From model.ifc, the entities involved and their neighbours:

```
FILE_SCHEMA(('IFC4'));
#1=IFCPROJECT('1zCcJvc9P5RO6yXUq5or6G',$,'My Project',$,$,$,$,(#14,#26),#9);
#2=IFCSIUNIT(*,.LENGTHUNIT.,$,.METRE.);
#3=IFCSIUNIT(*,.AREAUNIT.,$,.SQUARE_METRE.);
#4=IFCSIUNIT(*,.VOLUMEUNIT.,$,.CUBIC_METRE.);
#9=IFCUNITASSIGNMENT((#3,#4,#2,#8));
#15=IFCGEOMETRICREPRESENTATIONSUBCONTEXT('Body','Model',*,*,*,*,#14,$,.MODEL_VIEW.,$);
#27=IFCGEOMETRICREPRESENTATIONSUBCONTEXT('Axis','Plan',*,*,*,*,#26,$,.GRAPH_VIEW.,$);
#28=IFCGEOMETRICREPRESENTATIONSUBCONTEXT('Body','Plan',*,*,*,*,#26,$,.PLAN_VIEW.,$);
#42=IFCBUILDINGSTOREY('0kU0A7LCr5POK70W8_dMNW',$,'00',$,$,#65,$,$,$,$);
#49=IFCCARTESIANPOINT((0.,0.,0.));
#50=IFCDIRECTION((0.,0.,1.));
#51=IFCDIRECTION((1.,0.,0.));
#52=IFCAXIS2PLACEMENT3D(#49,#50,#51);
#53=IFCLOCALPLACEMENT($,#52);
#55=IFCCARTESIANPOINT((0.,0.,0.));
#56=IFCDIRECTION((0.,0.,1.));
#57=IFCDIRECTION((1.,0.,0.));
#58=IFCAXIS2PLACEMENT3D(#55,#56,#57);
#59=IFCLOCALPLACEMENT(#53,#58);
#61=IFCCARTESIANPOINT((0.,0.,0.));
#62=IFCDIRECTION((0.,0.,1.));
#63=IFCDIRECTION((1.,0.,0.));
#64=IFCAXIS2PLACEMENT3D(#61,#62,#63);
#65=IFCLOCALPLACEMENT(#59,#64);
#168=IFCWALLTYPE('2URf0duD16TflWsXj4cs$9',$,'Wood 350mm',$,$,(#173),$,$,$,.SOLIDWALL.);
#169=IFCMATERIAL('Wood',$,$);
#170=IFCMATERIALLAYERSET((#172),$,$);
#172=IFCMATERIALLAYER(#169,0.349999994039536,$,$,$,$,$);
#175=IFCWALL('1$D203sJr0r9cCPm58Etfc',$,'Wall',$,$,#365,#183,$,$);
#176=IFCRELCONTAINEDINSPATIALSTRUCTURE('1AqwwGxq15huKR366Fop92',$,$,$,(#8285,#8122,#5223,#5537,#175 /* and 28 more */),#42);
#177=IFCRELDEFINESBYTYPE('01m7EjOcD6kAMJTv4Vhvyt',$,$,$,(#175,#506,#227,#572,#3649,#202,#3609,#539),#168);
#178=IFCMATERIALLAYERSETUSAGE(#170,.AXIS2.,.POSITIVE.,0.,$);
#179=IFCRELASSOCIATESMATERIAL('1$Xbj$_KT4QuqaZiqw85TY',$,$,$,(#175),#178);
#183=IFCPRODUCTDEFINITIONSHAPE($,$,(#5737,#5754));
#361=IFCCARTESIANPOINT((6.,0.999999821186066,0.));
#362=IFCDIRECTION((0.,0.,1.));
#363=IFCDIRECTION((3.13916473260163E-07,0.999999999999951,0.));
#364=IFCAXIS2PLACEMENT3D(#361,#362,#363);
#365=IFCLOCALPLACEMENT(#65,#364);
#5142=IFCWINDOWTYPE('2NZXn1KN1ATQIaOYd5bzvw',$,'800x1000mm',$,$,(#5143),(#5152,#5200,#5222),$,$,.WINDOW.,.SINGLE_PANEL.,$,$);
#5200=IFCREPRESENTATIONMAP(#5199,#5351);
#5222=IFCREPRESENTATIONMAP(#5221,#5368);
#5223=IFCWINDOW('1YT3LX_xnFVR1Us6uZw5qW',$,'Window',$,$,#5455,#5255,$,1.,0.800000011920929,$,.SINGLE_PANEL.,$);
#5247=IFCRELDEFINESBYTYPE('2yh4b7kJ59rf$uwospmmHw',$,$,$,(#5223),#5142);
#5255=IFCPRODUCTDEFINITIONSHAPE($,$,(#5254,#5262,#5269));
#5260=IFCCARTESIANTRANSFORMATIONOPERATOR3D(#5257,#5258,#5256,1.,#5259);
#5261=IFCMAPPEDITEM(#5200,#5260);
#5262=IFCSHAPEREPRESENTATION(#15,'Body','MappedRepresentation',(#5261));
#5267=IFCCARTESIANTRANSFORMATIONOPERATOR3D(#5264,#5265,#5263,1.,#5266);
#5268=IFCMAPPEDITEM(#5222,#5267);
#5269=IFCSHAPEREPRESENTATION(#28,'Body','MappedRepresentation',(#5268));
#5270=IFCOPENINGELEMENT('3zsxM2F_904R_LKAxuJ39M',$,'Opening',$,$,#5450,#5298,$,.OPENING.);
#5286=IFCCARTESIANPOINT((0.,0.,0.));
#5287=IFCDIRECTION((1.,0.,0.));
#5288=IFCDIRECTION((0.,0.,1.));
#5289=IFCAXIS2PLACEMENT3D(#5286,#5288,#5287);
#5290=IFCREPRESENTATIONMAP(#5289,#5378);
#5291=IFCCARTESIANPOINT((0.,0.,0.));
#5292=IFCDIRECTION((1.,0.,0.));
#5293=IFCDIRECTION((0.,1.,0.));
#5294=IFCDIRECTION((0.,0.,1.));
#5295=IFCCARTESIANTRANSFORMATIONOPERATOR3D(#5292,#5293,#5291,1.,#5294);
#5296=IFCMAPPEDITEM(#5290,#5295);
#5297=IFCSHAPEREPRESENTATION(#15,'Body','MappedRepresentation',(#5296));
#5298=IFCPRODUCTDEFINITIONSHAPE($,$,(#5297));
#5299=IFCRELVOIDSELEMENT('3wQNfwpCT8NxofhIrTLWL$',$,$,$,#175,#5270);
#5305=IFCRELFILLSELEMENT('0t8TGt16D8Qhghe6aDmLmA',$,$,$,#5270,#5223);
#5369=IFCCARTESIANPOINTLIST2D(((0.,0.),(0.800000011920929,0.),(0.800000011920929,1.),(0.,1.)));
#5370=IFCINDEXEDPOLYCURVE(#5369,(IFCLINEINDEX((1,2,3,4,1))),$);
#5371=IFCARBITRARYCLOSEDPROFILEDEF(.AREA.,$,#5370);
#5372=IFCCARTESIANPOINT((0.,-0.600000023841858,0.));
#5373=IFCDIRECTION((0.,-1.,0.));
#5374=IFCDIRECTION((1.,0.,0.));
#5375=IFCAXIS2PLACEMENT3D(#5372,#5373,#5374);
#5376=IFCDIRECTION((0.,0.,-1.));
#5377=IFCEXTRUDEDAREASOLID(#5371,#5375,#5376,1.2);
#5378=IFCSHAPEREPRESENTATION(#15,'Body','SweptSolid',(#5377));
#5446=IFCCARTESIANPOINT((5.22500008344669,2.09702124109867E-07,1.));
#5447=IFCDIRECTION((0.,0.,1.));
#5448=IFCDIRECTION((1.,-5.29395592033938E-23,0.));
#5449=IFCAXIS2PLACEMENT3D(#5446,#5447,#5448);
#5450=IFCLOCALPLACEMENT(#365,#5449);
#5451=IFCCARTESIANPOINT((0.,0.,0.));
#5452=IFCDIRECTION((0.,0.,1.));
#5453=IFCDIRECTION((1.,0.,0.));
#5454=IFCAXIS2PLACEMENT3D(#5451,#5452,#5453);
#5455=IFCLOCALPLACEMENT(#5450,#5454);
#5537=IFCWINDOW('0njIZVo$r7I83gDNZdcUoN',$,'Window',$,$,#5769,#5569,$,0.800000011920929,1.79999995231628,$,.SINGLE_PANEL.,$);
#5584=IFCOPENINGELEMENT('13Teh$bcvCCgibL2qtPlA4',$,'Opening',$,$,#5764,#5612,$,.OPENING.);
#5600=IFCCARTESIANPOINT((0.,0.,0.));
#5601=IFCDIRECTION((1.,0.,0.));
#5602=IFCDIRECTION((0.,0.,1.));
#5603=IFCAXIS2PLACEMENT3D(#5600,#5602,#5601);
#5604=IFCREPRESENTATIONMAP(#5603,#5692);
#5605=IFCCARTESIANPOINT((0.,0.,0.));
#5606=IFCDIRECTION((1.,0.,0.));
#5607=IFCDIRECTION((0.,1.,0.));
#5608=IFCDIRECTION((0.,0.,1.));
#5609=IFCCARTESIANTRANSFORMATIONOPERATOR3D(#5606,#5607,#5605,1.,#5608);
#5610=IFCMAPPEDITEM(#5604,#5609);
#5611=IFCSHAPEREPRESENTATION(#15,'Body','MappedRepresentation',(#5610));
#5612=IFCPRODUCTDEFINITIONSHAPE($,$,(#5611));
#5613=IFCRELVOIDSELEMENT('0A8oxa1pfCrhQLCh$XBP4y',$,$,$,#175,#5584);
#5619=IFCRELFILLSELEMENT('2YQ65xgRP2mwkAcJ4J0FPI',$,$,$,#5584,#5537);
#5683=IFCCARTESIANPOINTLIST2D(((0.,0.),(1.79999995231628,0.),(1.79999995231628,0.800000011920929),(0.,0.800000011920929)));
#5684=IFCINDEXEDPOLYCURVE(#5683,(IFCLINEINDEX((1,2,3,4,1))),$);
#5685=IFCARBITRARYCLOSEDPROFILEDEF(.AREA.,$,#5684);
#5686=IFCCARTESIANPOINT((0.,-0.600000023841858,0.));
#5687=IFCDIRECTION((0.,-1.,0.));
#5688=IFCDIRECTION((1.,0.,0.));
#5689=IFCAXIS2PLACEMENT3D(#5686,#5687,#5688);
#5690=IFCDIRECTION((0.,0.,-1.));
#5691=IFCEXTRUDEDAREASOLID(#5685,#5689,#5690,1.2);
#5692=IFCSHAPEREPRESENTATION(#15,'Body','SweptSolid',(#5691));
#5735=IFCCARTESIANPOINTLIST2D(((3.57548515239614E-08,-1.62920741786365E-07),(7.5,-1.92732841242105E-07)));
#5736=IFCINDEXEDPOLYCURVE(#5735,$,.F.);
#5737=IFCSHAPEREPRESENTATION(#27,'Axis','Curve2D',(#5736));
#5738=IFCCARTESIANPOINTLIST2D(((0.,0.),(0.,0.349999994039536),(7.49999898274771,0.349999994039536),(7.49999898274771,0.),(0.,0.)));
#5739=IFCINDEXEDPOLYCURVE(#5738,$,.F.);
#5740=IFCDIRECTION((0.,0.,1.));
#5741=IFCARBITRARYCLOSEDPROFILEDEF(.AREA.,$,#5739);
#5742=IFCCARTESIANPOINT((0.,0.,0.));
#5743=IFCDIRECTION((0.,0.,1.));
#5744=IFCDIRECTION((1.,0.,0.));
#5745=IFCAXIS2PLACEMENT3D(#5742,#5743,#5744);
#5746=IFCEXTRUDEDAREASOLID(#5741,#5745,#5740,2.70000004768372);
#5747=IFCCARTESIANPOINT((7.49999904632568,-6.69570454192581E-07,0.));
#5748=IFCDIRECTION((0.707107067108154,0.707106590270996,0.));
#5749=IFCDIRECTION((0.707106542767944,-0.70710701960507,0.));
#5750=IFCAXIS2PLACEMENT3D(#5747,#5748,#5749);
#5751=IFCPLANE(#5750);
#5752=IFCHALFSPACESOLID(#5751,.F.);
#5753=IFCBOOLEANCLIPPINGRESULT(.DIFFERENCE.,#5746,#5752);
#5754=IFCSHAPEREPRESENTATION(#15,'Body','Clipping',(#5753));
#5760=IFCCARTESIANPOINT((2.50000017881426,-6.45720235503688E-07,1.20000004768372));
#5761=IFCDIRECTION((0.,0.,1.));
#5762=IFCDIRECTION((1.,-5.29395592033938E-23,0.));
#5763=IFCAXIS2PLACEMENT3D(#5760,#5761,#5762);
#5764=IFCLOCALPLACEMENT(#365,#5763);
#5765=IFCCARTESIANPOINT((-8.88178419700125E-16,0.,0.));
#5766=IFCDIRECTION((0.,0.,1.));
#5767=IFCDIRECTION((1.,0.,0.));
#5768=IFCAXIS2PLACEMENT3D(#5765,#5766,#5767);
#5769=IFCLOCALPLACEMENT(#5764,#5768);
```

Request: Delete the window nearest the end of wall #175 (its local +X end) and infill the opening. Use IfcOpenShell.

```python
import ifcopenshell
import ifcopenshell.api.feature
import ifcopenshell.api.root
import ifcopenshell.geom
import ifcopenshell.util.shape

model = ifcopenshell.open("model.ifc")
settings = ifcopenshell.geom.settings()


def volume(element):
    """Net volume in cubic metres, openings subtracted."""
    shape = ifcopenshell.geom.create_shape(settings, element)
    return ifcopenshell.util.shape.get_volume(shape.geometry)


window = model.by_id(5223)
opening = window.FillsVoids[0].RelatingOpeningElement
wall = opening.VoidsElements[0].RelatingBuildingElement
before = volume(wall)

ifcopenshell.api.root.remove_product(model, product=window)
ifcopenshell.api.feature.remove_feature(model, feature=opening)

after = volume(wall)

print(f"wall volume {before:.3f} -> {after:.3f} m3")

model.write("model_v2.ifc")
```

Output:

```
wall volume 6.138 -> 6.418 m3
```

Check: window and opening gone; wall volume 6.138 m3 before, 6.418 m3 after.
